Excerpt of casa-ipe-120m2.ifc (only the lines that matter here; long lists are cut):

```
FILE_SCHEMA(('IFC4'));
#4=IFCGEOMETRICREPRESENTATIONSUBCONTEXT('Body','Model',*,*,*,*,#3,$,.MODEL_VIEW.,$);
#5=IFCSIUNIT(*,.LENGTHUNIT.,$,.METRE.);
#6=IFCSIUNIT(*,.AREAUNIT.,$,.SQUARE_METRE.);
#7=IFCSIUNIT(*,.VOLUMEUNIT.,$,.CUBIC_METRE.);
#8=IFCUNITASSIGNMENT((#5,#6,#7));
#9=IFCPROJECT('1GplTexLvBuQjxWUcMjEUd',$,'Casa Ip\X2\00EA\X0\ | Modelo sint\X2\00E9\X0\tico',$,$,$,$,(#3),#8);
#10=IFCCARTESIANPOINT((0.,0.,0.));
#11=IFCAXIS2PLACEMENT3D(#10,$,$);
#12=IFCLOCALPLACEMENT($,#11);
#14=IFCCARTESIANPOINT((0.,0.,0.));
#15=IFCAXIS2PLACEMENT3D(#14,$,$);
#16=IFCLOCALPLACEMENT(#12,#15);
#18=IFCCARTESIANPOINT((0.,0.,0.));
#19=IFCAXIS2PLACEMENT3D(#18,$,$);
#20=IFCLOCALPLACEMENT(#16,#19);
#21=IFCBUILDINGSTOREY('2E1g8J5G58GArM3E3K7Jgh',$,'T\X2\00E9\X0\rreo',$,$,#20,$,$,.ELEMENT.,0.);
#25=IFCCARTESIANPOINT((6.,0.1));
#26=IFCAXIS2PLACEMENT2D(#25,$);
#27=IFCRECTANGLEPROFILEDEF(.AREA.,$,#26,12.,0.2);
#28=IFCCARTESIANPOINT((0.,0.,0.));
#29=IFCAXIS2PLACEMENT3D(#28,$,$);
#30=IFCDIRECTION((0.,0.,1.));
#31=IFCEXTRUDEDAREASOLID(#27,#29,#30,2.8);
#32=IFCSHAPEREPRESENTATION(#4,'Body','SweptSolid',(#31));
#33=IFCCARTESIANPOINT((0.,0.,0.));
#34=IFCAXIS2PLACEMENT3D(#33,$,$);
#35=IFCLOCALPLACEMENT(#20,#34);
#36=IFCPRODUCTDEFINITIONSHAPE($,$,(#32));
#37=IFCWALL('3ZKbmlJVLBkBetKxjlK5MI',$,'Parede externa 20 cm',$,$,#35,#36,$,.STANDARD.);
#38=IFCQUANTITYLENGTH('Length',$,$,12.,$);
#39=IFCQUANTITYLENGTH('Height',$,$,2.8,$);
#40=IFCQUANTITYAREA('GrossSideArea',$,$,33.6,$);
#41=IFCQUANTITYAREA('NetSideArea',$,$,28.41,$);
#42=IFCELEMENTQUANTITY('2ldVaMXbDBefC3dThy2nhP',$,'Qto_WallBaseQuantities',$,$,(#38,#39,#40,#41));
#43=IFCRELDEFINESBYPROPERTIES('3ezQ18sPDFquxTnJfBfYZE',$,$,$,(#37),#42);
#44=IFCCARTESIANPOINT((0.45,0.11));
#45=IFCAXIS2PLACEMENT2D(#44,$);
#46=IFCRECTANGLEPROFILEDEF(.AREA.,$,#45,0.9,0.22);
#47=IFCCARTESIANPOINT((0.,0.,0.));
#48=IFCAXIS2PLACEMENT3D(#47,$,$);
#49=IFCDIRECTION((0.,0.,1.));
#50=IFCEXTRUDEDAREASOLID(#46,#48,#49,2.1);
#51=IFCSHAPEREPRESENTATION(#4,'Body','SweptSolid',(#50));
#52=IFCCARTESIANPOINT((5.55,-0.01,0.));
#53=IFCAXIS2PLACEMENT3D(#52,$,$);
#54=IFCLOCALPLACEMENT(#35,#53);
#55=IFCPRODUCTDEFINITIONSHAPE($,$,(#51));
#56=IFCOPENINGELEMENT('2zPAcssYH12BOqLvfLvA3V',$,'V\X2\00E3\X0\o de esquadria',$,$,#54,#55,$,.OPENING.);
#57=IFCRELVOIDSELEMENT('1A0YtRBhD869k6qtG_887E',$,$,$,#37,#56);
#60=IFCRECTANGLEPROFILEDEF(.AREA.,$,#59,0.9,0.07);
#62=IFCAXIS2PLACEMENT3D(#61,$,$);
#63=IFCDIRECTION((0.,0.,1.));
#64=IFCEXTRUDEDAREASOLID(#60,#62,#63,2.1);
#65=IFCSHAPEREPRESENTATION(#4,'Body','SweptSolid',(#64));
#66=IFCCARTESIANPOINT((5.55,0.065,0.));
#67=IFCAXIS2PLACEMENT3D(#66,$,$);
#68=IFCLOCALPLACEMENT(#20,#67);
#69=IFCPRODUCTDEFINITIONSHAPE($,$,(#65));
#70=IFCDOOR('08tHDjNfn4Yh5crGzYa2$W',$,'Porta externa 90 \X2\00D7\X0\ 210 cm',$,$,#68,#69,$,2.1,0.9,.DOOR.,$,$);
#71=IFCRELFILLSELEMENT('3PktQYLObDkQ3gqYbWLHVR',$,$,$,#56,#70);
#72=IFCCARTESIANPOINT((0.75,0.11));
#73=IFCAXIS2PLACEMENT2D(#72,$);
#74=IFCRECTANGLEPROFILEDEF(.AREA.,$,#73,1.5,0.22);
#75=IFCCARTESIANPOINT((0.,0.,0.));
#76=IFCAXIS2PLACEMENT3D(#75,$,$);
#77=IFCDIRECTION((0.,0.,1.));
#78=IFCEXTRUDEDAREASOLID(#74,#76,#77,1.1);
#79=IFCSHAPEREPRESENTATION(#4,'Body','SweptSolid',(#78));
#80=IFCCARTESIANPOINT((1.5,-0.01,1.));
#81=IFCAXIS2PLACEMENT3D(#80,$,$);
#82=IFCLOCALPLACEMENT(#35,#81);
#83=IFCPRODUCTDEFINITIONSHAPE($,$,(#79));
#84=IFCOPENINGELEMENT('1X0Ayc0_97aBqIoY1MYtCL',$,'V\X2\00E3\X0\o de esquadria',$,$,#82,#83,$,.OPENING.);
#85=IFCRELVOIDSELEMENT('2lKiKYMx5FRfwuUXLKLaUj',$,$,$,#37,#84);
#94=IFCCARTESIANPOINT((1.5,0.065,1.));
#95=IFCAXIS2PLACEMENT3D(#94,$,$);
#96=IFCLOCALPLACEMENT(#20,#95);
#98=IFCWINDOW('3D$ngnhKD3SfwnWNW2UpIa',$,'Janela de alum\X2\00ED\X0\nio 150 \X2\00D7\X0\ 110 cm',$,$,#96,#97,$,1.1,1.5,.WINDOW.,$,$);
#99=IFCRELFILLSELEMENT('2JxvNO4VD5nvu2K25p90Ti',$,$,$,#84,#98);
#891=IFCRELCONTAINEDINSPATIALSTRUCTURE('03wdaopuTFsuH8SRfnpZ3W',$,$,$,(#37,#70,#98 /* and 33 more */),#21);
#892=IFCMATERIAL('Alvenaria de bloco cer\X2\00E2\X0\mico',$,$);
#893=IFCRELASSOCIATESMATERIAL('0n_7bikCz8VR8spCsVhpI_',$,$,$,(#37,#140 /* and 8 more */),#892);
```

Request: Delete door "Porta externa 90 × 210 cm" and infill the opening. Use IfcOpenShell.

```python
import ifcopenshell
import ifcopenshell.api.feature
import ifcopenshell.api.pset
import ifcopenshell.api.root
import ifcopenshell.geom
import ifcopenshell.util.element
import ifcopenshell.util.shape
import ifcopenshell.util.unit

model = ifcopenshell.open("casa-ipe-120m2.ifc")
area_scale = ifcopenshell.util.unit.calculate_unit_scale(model, "AREAUNIT")
settings = ifcopenshell.geom.settings()


def volume(element):
    """Net volume in cubic metres, openings subtracted."""
    shape = ifcopenshell.geom.create_shape(settings, element)
    return ifcopenshell.util.shape.get_volume(shape.geometry)


door = model.by_id(70)
opening = door.FillsVoids[0].RelatingOpeningElement
wall = opening.VoidsElements[0].RelatingBuildingElement
before = volume(wall)

ifcopenshell.api.root.remove_product(model, product=door)
ifcopenshell.api.feature.remove_feature(model, feature=opening)

after = volume(wall)
thickness = 0.2  # wall thickness in metres

# Update the wall's stored quantities.
qto = model.by_id(ifcopenshell.util.element.get_pset(wall, "Qto_WallBaseQuantities", should_inherit=False)["id"])
ifcopenshell.api.pset.edit_qto(model, qto=qto, properties={"NetSideArea": after / thickness / area_scale})

print(f"wall volume {before:.3f} -> {after:.3f} m3")

model.write("casa-ipe-120m2_edited.ifc")
```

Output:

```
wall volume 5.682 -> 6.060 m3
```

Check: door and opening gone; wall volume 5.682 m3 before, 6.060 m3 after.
